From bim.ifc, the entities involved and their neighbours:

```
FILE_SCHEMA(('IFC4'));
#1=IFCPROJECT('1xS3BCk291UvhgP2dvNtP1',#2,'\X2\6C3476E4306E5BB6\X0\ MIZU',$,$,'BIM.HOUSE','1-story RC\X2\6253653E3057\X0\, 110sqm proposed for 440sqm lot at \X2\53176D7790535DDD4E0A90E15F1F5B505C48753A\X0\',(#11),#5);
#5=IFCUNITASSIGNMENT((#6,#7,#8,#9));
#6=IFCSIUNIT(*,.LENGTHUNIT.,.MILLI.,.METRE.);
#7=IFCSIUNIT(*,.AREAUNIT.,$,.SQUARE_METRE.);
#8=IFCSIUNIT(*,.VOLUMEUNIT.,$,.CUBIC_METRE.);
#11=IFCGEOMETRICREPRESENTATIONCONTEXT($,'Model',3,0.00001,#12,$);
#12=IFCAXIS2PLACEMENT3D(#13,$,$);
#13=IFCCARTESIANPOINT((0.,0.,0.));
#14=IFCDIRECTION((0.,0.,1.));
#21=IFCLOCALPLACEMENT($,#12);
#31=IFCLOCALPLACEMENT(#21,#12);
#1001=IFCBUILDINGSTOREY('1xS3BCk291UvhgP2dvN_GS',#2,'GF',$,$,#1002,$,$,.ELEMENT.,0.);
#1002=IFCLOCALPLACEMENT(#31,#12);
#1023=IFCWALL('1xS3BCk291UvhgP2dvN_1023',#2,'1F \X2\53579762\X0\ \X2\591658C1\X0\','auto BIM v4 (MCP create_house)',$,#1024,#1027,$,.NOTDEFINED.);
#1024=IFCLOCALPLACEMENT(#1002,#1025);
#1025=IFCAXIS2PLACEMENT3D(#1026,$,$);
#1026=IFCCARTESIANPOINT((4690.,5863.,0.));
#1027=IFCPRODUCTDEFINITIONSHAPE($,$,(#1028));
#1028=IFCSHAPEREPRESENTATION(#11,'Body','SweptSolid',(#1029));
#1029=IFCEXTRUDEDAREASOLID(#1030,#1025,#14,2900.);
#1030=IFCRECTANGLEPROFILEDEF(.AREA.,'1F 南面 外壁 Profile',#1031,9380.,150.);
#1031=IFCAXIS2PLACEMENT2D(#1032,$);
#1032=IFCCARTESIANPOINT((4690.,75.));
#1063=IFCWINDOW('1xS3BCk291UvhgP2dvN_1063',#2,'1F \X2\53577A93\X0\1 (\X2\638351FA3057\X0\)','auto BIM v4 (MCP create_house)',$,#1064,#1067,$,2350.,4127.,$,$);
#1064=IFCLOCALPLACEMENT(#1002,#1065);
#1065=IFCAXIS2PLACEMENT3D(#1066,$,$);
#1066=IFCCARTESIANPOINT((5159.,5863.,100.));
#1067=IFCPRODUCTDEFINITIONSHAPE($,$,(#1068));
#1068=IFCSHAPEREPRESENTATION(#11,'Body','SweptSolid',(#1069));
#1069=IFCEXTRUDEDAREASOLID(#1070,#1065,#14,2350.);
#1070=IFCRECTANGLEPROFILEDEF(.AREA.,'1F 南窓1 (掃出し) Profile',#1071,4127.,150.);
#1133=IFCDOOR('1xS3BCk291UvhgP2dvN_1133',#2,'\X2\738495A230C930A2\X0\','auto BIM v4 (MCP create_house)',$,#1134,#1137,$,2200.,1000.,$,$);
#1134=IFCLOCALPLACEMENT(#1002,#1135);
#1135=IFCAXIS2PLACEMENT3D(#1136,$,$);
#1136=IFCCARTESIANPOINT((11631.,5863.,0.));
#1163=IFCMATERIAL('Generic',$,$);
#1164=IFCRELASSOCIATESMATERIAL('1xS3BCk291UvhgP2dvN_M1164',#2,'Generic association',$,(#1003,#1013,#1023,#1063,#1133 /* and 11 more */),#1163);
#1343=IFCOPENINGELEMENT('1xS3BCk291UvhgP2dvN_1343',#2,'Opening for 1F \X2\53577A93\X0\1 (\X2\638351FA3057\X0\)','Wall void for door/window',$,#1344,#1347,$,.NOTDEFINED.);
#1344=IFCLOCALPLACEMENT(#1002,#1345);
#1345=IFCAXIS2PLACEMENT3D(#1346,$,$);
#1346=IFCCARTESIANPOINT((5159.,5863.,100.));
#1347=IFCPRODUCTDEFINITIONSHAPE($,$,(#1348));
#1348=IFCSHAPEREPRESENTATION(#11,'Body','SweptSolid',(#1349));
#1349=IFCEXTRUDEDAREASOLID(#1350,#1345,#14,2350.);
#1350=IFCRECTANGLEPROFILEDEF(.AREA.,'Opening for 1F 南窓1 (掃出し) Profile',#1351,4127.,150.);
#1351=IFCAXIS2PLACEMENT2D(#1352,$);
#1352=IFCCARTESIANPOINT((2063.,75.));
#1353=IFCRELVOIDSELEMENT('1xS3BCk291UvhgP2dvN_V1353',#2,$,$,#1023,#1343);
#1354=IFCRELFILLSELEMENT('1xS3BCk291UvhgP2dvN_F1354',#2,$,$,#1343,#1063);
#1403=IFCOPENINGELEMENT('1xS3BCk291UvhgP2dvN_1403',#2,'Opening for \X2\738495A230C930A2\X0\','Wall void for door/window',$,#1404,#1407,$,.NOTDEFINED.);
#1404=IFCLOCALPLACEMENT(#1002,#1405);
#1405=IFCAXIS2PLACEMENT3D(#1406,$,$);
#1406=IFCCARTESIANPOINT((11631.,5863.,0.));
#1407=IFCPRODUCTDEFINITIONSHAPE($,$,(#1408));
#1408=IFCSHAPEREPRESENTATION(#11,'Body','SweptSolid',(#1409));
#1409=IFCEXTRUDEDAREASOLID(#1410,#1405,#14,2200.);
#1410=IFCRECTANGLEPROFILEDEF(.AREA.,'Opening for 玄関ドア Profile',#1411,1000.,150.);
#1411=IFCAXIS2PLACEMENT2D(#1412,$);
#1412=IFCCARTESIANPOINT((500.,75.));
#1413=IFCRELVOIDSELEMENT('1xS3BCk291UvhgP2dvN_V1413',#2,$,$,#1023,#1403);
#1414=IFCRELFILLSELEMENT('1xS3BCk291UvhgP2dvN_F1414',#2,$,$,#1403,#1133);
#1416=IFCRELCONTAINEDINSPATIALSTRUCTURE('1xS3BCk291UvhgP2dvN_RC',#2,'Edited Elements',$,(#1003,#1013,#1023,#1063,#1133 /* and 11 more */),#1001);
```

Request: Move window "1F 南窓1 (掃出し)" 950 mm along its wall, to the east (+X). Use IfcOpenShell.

```python
import ifcopenshell
import ifcopenshell.api.geometry
import ifcopenshell.util.placement
import ifcopenshell.util.unit

model = ifcopenshell.open("bim.ifc")
unit_scale = ifcopenshell.util.unit.calculate_unit_scale(model)

window = model.by_id(1063)
opening = window.FillsVoids[0].RelatingOpeningElement
wall = opening.VoidsElements[0].RelatingBuildingElement

wall_matrix = ifcopenshell.util.placement.get_local_placement(wall.ObjectPlacement)
shift = wall_matrix[:3, 0] * 0.95 / unit_scale
before = ifcopenshell.util.placement.get_local_placement(window.ObjectPlacement)[:3, 3].copy()

# The window is not placed relative to its opening, so move both.
for product in (opening, window):
    matrix = ifcopenshell.util.placement.get_local_placement(product.ObjectPlacement)
    matrix[:3, 3] += shift
    ifcopenshell.api.geometry.edit_object_placement(model, product=product, matrix=matrix, is_si=False)

after = ifcopenshell.util.placement.get_local_placement(window.ObjectPlacement)[:3, 3]
print("window moved by", (after - before).round(3) + 0.0)

model.write("bim_rev.ifc")
```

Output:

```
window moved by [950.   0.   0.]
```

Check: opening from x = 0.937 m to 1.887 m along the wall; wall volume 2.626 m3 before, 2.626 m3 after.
